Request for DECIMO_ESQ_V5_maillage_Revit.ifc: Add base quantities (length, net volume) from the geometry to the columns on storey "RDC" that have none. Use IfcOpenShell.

First a look at what the model holds.

```python
import ifcopenshell
import ifcopenshell.util.element
import ifcopenshell.util.unit

model = ifcopenshell.open("DECIMO_ESQ_V5_maillage_Revit.ifc")
print(model.schema)
for unit_type in ("LENGTHUNIT", "AREAUNIT", "VOLUMEUNIT"):
    print(unit_type, ifcopenshell.util.unit.calculate_unit_scale(model, unit_type))
storey = next(s for s in model.by_type("IfcBuildingStorey") if s.Name == "RDC")
columns = [e for e in ifcopenshell.util.element.get_decomposition(storey) if e.is_a("IfcColumn")]
for e in sorted(columns, key=lambda e: e.id()):
    print(e.id(), e.is_a(), e.Name, list(ifcopenshell.util.element.get_psets(e, qtos_only=True)), sep=" | ")
```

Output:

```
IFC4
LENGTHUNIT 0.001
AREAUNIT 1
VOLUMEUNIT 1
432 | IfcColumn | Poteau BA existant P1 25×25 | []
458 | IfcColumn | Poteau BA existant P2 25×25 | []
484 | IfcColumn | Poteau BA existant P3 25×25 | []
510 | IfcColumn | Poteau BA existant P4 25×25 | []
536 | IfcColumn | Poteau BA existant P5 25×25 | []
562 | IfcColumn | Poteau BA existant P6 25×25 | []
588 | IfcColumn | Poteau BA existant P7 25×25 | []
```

```python
import ifcopenshell
import ifcopenshell.api.pset
import ifcopenshell.geom
import ifcopenshell.util.element
import ifcopenshell.util.shape
import ifcopenshell.util.unit

model = ifcopenshell.open("DECIMO_ESQ_V5_maillage_Revit.ifc")
unit_scale = ifcopenshell.util.unit.calculate_unit_scale(model)
volume_scale = ifcopenshell.util.unit.calculate_unit_scale(model, "VOLUMEUNIT")
settings = ifcopenshell.geom.settings()

storey = next(s for s in model.by_type("IfcBuildingStorey") if s.Name == "RDC")
columns = [e for e in ifcopenshell.util.element.get_decomposition(storey) if e.is_a("IfcColumn")]

for e in sorted(columns, key=lambda e: e.id()):
    if ifcopenshell.util.element.get_psets(e, qtos_only=True, should_inherit=False):
        continue
    # Geometry comes back in metres, in the element's own axes.
    shape = ifcopenshell.geom.create_shape(settings, e)
    values = {
        "Length": ifcopenshell.util.shape.get_z(shape.geometry) / unit_scale,
        "NetVolume": ifcopenshell.util.shape.get_volume(shape.geometry) / volume_scale,
    }
    qto = ifcopenshell.api.pset.add_qto(model, product=e, name="Qto_ColumnBaseQuantities")
    ifcopenshell.api.pset.edit_qto(model, qto=qto, properties=values)
    print(e.id(), {k: round(v, 3) for k, v in values.items()})

model.write("DECIMO_ESQ_V5_maillage_Revit-out.ifc")
```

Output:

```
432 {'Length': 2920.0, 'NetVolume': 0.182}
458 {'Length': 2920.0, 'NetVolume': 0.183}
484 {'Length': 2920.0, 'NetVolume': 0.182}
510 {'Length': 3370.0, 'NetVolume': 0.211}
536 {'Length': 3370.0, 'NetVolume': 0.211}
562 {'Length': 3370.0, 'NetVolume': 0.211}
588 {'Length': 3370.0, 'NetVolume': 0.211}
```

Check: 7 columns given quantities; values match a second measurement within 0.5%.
